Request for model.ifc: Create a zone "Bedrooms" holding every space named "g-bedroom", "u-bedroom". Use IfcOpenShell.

First a look at what the model holds.

```python
import ifcopenshell

model = ifcopenshell.open("model.ifc")
print(model.schema)
seen = {}
for space in model.by_type("IfcSpace"):
    seen[space.LongName] = seen.get(space.LongName, 0) + 1
for name, count in sorted(seen.items(), key=str):
    print(count, "x", name)
print("zones:", [z.Name for z in model.by_type("IfcZone")][:20])
```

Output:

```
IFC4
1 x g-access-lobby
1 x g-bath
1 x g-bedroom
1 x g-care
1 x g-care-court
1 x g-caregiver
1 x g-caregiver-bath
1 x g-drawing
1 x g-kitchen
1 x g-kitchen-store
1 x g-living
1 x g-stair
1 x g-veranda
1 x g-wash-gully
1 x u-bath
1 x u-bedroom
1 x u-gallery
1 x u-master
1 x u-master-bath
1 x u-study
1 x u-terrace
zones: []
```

```python
import ifcopenshell
import ifcopenshell.api.group
import ifcopenshell.api.root

model = ifcopenshell.open("model.ifc")

names = {"g-bedroom", "u-bedroom"}
spaces = [s for s in model.by_type("IfcSpace") if s.LongName in names]

zone = ifcopenshell.api.root.create_entity(model, ifc_class="IfcZone", name="Bedrooms")
ifcopenshell.api.group.assign_group(model, products=spaces, group=zone)
print(len(spaces), "spaces in", zone.Name)

model.write("model_edited.ifc")
```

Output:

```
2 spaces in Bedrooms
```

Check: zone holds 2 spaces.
